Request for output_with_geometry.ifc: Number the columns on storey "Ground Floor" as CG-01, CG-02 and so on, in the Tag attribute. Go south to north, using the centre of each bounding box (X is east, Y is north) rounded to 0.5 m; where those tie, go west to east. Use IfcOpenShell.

First a look at what the model holds.

```python
import ifcopenshell
import ifcopenshell.util.element
import ifcopenshell.util.placement

model = ifcopenshell.open("output_with_geometry.ifc")
print(model.schema)
storey = next(s for s in model.by_type("IfcBuildingStorey") if s.Name == "Ground Floor")
columns = [e for e in ifcopenshell.util.element.get_decomposition(storey) if e.is_a("IfcColumn")]
for e in sorted(columns, key=lambda e: e.id()):
    origin = ifcopenshell.util.placement.get_local_placement(e.ObjectPlacement)[:3, 3]
    print(e.id(), e.Tag, e.Name, origin.round(2) + 0.0, sep=" | ")
```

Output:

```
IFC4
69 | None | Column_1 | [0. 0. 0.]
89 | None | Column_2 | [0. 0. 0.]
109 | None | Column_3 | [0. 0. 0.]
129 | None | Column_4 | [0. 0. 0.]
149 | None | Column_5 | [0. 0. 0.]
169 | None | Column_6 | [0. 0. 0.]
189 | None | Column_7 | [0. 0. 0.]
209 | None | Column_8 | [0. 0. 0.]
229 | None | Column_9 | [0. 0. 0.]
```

```python
import ifcopenshell
import ifcopenshell.geom
import ifcopenshell.util.element
import ifcopenshell.util.shape

model = ifcopenshell.open("output_with_geometry.ifc")
settings = ifcopenshell.geom.settings()
settings.set("use-world-coords", True)


def centre(element):
    shape = ifcopenshell.geom.create_shape(settings, element)
    return ifcopenshell.util.shape.get_bbox_centroid(shape.geometry)


storey = next(s for s in model.by_type("IfcBuildingStorey") if s.Name == "Ground Floor")
columns = [e for e in ifcopenshell.util.element.get_decomposition(storey) if e.is_a("IfcColumn")]

# Insertion points can sit at a corner or the storey origin, so sort by the geometry (in metres).
centres = {e: centre(e) for e in columns}
columns.sort(key=lambda e: (round(centres[e][1] / 0.5), centres[e][0]))

for i, e in enumerate(columns, start=1):
    number = f"CG-{i:02d}"
    e.Tag = number
    print(e.id(), number)

model.write("output_with_geometry_v2.ifc")
```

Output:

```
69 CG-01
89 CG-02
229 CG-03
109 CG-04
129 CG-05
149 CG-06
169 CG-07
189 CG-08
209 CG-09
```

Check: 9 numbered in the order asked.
